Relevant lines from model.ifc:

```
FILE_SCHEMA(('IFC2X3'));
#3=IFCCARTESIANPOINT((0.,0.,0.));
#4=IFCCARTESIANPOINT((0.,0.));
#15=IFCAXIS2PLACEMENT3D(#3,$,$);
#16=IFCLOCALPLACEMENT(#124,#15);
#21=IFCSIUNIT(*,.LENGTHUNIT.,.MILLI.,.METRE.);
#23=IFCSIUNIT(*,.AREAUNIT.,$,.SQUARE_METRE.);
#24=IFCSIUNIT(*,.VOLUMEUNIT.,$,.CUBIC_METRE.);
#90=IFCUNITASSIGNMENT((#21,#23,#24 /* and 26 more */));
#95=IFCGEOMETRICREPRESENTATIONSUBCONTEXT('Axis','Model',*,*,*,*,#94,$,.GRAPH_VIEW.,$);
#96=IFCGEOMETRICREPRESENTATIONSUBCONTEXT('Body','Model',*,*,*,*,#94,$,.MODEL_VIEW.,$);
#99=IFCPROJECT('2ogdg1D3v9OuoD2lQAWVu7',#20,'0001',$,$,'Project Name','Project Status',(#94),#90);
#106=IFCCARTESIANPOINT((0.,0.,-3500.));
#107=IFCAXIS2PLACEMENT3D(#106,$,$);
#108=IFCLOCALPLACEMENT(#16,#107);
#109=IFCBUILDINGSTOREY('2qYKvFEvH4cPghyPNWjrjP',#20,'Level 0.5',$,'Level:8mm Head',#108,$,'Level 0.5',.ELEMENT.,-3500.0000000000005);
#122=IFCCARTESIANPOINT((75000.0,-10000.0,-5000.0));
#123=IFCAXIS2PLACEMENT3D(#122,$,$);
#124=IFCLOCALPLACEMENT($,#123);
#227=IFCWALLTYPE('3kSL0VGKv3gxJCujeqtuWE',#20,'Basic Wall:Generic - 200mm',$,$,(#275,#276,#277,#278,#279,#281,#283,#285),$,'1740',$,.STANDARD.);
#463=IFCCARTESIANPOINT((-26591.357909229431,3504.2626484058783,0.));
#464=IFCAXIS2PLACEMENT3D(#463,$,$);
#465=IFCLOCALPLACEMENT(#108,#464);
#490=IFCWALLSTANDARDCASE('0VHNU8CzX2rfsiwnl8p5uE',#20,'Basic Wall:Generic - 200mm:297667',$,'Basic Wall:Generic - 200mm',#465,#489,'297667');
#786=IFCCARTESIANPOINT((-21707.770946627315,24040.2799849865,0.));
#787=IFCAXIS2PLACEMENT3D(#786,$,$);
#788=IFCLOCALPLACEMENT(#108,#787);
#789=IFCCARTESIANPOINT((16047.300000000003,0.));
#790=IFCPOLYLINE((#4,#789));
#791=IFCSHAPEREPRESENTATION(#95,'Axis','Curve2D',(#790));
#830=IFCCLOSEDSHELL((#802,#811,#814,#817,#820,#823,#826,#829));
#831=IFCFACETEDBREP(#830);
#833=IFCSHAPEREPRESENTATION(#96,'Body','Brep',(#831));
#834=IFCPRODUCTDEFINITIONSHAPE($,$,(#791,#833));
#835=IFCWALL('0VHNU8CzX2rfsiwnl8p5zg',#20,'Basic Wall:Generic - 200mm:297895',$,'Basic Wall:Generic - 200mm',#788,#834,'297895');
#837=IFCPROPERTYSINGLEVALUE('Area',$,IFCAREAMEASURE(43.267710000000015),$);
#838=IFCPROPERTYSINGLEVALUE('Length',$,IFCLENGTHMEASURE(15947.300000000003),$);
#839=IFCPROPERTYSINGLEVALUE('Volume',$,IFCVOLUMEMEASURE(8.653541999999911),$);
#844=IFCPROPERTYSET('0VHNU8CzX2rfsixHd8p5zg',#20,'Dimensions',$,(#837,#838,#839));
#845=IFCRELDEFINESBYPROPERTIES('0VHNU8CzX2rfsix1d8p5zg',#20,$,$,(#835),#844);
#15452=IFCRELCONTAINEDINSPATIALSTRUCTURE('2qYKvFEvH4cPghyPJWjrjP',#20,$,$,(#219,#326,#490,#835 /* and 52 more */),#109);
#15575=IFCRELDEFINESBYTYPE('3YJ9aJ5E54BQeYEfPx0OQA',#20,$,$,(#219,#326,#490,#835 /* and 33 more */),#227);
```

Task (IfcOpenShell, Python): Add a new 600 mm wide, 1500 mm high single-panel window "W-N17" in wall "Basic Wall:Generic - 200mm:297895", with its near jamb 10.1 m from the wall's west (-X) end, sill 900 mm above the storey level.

```python
import numpy as np
import ifcopenshell
import ifcopenshell.api.feature
import ifcopenshell.api.geometry
import ifcopenshell.api.pset
import ifcopenshell.api.root
import ifcopenshell.api.spatial
import ifcopenshell.api.type
import ifcopenshell.geom
import ifcopenshell.util.element
import ifcopenshell.util.placement
import ifcopenshell.util.representation
import ifcopenshell.util.shape
import ifcopenshell.util.unit

model = ifcopenshell.open("model.ifc")
unit_scale = ifcopenshell.util.unit.calculate_unit_scale(model)
area_scale = ifcopenshell.util.unit.calculate_unit_scale(model, "AREAUNIT")
volume_scale = ifcopenshell.util.unit.calculate_unit_scale(model, "VOLUMEUNIT")
settings = ifcopenshell.geom.settings()


def volume(element):
    """Net volume in cubic metres, openings subtracted."""
    shape = ifcopenshell.geom.create_shape(settings, element)
    return ifcopenshell.util.shape.get_volume(shape.geometry)


wall = model.by_guid("0VHNU8CzX2rfsiwnl8p5zg")
storey = ifcopenshell.util.element.get_container(wall, ifc_class="IfcBuildingStorey")
context = ifcopenshell.util.representation.get_context(model, "Model", "Body", "MODEL_VIEW")
before = volume(wall)

width, height, from_end, sill = 0.6, 1.5, 10.1, 0.9  # metres

# The wall runs along its own X axis, and the end named is its -X end.
wall_shape = ifcopenshell.geom.create_shape(settings, wall)
x, y, z = ifcopenshell.util.shape.get_vertices(wall_shape.geometry).T
start = x.min() + from_end
face, thickness = float(y.min()), float(y.max() - y.min())
wall_matrix = ifcopenshell.util.placement.get_local_placement(wall.ObjectPlacement)
level = ifcopenshell.util.placement.get_local_placement(storey.ObjectPlacement)[2, 3]


def in_wall(x, y):
    """Placement at x, y metres in the wall's axes, at sill height."""
    matrix = wall_matrix.copy()
    matrix[:, 3] = wall_matrix @ np.array([x / unit_scale, y / unit_scale, 0.0, 1.0])
    matrix[2, 3] = level + sill / unit_scale
    return matrix


# Opening: a box that overshoots both wall faces by 50 mm.
opening = ifcopenshell.api.root.create_entity(model, ifc_class="IfcOpeningElement")
box = ifcopenshell.api.geometry.add_wall_representation(
    model, context=context, length=width, height=height, thickness=thickness + 0.1
)
ifcopenshell.api.geometry.assign_representation(model, product=opening, representation=box)
ifcopenshell.api.geometry.edit_object_placement(model, product=opening, matrix=in_wall(start, face - 0.05), is_si=False)
ifcopenshell.api.feature.add_feature(model, feature=opening, element=wall)

window = ifcopenshell.api.root.create_entity(model, ifc_class="IfcWindow", name="W-N17")
window.OverallWidth, window.OverallHeight = width / unit_scale, height / unit_scale
body = ifcopenshell.api.geometry.add_window_representation(
    model,
    context=context,
    overall_width=window.OverallWidth,
    overall_height=window.OverallHeight,
    partition_type="SINGLE_PANEL",
)
ifcopenshell.api.geometry.assign_representation(model, product=window, representation=body)
ifcopenshell.api.spatial.assign_container(model, products=[window], relating_structure=storey)
fills = ifcopenshell.api.feature.add_filling(model, opening=opening, element=window)
fills.OwnerHistory = window.OwnerHistory  # required in IFC2X3

# IFC2X3 keeps the operation on the window style.
style = ifcopenshell.api.root.create_entity(model, ifc_class="IfcWindowStyle", name="W-N17")
style.OperationType, style.ConstructionType = "SINGLE_PANEL", "NOTDEFINED"
style.ParameterTakesPrecedence = style.Sizeable = False
ifcopenshell.api.type.assign_type(model, related_objects=[window], relating_type=style)

# Centre the window in the wall's thickness.
ifcopenshell.api.geometry.edit_object_placement(model, product=window, matrix=in_wall(start, face), is_si=False)
window_shape = ifcopenshell.geom.create_shape(settings, window)
depth = ifcopenshell.util.shape.get_vertices(window_shape.geometry)[:, 1]
offset = face + thickness / 2 - (depth.min() + depth.max()) / 2
ifcopenshell.api.geometry.edit_object_placement(model, product=window, matrix=in_wall(start, offset), is_si=False)

after = volume(wall)

# Update the wall's stored quantities.
pset = model.by_id(ifcopenshell.util.element.get_pset(wall, "Dimensions", should_inherit=False)["id"])
ifcopenshell.api.pset.edit_pset(model, pset=pset, properties={
    "Area": model.create_entity("IfcAreaMeasure", after / thickness / area_scale),
    "Volume": model.create_entity("IfcVolumeMeasure", after / volume_scale),
})

print(f"wall volume {before:.3f} -> {after:.3f} m3")

model.write("model_edited.ifc")
```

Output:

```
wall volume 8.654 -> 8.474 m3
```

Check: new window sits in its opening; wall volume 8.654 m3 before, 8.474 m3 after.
